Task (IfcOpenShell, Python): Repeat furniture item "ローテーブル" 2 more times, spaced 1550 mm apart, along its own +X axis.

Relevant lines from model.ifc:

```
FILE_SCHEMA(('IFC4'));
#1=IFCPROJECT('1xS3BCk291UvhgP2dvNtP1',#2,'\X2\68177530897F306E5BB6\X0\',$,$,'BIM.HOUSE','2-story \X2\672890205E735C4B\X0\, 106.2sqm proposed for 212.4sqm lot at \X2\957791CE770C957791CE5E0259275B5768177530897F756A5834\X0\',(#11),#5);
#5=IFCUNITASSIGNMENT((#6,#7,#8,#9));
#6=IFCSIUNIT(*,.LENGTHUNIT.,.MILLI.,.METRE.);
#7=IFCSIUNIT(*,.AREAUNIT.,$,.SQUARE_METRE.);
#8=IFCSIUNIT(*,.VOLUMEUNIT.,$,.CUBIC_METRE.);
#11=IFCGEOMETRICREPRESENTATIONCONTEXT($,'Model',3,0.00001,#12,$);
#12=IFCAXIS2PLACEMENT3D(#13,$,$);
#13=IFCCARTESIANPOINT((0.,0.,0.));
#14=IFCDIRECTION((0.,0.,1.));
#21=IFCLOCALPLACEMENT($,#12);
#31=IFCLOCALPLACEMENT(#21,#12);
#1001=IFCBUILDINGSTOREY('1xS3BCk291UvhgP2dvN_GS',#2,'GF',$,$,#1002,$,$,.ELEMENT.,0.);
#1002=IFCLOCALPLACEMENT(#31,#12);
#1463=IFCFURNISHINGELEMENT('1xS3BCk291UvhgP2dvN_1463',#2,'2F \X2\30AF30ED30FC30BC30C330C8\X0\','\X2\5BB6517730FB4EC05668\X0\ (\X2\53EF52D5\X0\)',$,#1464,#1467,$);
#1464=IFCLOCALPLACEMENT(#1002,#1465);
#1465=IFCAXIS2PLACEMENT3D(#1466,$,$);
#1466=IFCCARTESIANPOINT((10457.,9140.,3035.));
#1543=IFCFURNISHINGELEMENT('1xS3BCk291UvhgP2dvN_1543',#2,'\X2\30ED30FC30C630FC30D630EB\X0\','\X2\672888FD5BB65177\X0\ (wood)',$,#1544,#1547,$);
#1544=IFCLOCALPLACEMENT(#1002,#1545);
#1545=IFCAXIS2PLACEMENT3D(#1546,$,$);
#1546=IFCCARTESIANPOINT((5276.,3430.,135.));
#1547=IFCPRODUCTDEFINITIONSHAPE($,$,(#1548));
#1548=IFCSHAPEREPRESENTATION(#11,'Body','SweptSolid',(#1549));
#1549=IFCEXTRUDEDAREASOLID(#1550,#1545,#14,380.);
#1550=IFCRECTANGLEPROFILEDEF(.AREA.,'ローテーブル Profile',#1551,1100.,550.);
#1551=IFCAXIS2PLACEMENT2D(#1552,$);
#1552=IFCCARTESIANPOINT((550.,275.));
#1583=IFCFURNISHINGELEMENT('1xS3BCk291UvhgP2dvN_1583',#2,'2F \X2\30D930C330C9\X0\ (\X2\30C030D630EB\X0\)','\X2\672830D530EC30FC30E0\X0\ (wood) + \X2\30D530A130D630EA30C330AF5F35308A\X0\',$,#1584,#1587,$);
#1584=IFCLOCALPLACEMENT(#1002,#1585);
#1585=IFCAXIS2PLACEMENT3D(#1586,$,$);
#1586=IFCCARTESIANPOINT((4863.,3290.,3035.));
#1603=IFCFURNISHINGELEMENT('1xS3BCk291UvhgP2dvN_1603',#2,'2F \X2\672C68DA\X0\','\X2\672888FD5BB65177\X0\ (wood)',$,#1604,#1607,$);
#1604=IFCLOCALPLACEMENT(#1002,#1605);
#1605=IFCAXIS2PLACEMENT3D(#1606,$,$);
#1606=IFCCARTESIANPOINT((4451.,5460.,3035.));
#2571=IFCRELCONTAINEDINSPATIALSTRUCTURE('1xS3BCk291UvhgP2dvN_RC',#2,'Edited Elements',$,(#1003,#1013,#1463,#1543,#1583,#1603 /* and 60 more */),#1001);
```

```python
import ifcopenshell
import ifcopenshell.api.geometry
import ifcopenshell.api.root
import ifcopenshell.util.element
import ifcopenshell.util.placement

model = ifcopenshell.open("model.ifc")


def reuse_history(source, copy):
    """copy_class also copies each property set's owner history, people and application; keep the originals."""
    for rel in copy.IsDefinedBy:
        if rel.is_a("IfcRelDefinesByProperties") and (history := rel.RelatingPropertyDefinition.OwnerHistory):
            rel.RelatingPropertyDefinition.OwnerHistory = source.OwnerHistory
            ifcopenshell.util.element.remove_deep2(model, history)


source = model.by_guid("1xS3BCk291UvhgP2dvN_1543")
base = ifcopenshell.util.placement.get_local_placement(source.ObjectPlacement)
step = base[:3, 0] * 1550.0

for i in range(1, 3):
    copy = ifcopenshell.api.root.copy_class(model, product=source)
    copy.Representation = ifcopenshell.util.element.copy_deep(
        model, source.Representation, exclude=["IfcGeometricRepresentationContext", "IfcRepresentationMap"]
    )
    reuse_history(source, copy)
    matrix = base.copy()
    matrix[:3, 3] += i * step
    print("added at", matrix[:3, 3].round(3) + 0.0)
    ifcopenshell.api.geometry.edit_object_placement(model, product=copy, matrix=matrix, is_si=False)

model.write("model_edited.ifc")
```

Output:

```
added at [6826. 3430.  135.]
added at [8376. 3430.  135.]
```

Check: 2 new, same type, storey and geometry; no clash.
